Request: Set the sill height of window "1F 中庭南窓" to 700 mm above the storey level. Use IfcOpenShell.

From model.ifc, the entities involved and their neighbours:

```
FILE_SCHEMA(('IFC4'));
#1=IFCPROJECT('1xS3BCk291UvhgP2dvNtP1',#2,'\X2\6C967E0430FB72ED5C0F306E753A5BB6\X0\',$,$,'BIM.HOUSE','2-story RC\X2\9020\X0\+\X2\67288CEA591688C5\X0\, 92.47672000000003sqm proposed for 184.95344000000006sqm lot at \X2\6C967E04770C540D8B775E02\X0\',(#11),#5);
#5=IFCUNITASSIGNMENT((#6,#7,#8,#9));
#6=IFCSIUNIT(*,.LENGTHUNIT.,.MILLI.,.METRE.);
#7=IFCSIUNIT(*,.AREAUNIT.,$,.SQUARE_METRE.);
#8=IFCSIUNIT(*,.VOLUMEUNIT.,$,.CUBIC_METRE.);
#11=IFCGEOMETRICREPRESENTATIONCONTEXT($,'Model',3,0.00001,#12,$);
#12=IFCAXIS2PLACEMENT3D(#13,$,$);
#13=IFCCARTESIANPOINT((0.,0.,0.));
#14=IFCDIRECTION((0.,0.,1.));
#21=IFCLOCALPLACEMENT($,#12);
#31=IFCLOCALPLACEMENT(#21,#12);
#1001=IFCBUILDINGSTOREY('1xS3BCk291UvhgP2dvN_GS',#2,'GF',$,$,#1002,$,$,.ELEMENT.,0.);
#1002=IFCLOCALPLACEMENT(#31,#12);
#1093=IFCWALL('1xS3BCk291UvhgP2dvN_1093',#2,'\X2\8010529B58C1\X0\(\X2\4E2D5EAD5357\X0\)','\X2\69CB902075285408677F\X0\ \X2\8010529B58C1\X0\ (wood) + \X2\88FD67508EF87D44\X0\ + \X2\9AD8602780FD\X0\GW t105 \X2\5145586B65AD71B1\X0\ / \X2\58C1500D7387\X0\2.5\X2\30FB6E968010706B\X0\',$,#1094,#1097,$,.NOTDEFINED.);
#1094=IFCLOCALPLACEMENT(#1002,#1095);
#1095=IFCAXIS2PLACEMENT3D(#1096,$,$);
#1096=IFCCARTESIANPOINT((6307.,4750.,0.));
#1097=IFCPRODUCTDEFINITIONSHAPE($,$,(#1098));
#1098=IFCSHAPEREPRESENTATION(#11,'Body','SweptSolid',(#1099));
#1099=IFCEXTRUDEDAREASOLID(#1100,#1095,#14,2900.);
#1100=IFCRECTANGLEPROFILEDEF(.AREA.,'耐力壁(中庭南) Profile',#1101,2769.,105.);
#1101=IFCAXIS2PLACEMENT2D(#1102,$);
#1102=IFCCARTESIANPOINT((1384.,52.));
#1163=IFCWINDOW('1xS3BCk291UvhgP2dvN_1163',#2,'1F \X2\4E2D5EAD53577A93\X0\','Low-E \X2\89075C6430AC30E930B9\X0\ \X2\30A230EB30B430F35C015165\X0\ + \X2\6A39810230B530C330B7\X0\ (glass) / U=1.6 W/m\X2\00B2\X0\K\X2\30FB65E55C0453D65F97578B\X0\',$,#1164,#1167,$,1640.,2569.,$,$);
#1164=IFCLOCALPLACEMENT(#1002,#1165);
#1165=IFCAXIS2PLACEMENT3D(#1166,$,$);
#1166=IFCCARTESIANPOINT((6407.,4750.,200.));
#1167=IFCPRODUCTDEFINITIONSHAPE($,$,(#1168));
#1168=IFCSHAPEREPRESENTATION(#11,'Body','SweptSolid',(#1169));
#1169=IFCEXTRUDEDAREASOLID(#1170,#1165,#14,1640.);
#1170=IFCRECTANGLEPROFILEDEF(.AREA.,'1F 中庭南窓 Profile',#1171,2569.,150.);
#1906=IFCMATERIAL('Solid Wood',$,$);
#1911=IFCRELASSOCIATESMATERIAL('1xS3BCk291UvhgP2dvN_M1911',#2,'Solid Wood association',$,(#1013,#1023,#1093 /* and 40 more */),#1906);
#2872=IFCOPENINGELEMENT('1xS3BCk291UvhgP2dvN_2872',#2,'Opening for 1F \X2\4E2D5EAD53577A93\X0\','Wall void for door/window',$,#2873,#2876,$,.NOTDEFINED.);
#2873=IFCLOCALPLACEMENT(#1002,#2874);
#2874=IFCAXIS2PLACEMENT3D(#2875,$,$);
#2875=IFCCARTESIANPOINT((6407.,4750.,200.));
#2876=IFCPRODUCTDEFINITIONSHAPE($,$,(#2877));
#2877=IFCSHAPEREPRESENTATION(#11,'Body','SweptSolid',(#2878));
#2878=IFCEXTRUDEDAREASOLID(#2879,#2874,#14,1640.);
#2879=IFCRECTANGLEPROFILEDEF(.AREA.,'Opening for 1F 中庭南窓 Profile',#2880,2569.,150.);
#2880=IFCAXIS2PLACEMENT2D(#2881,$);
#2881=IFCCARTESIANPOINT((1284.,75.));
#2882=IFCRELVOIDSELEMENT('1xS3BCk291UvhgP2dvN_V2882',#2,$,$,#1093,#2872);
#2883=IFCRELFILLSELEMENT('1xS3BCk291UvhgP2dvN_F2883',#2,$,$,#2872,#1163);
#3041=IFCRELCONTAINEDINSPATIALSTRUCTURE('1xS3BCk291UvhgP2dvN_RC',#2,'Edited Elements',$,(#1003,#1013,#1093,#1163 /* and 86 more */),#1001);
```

```python
import numpy as np
import ifcopenshell
import ifcopenshell.api.geometry
import ifcopenshell.geom
import ifcopenshell.util.element
import ifcopenshell.util.placement
import ifcopenshell.util.shape
import ifcopenshell.util.unit

model = ifcopenshell.open("model.ifc")
unit_scale = ifcopenshell.util.unit.calculate_unit_scale(model)

window = model.by_id(1163)
opening = window.FillsVoids[0].RelatingOpeningElement
storey = ifcopenshell.util.element.get_container(window, ifc_class="IfcBuildingStorey")
level = ifcopenshell.util.placement.get_local_placement(storey.ObjectPlacement)[2, 3]

# The opening's origin need not be at the sill, so measure its lowest point.
shape = ifcopenshell.geom.create_shape(ifcopenshell.geom.settings(), opening)
bottom = ifcopenshell.util.shape.get_shape_bottom_elevation(shape, shape.geometry) / unit_scale
dz = level + 0.7 / unit_scale - bottom

shift = np.array([0.0, 0.0, dz])
# The window is not placed relative to its opening, so move both.
for product in (opening, window):
    matrix = ifcopenshell.util.placement.get_local_placement(product.ObjectPlacement)
    matrix[:3, 3] += shift
    ifcopenshell.api.geometry.edit_object_placement(model, product=product, matrix=matrix, is_si=False)

print(f"moved by {dz * unit_scale:+.3f} m")

model.write("model_v2.ifc")
```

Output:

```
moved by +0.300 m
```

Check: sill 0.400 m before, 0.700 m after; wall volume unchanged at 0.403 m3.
